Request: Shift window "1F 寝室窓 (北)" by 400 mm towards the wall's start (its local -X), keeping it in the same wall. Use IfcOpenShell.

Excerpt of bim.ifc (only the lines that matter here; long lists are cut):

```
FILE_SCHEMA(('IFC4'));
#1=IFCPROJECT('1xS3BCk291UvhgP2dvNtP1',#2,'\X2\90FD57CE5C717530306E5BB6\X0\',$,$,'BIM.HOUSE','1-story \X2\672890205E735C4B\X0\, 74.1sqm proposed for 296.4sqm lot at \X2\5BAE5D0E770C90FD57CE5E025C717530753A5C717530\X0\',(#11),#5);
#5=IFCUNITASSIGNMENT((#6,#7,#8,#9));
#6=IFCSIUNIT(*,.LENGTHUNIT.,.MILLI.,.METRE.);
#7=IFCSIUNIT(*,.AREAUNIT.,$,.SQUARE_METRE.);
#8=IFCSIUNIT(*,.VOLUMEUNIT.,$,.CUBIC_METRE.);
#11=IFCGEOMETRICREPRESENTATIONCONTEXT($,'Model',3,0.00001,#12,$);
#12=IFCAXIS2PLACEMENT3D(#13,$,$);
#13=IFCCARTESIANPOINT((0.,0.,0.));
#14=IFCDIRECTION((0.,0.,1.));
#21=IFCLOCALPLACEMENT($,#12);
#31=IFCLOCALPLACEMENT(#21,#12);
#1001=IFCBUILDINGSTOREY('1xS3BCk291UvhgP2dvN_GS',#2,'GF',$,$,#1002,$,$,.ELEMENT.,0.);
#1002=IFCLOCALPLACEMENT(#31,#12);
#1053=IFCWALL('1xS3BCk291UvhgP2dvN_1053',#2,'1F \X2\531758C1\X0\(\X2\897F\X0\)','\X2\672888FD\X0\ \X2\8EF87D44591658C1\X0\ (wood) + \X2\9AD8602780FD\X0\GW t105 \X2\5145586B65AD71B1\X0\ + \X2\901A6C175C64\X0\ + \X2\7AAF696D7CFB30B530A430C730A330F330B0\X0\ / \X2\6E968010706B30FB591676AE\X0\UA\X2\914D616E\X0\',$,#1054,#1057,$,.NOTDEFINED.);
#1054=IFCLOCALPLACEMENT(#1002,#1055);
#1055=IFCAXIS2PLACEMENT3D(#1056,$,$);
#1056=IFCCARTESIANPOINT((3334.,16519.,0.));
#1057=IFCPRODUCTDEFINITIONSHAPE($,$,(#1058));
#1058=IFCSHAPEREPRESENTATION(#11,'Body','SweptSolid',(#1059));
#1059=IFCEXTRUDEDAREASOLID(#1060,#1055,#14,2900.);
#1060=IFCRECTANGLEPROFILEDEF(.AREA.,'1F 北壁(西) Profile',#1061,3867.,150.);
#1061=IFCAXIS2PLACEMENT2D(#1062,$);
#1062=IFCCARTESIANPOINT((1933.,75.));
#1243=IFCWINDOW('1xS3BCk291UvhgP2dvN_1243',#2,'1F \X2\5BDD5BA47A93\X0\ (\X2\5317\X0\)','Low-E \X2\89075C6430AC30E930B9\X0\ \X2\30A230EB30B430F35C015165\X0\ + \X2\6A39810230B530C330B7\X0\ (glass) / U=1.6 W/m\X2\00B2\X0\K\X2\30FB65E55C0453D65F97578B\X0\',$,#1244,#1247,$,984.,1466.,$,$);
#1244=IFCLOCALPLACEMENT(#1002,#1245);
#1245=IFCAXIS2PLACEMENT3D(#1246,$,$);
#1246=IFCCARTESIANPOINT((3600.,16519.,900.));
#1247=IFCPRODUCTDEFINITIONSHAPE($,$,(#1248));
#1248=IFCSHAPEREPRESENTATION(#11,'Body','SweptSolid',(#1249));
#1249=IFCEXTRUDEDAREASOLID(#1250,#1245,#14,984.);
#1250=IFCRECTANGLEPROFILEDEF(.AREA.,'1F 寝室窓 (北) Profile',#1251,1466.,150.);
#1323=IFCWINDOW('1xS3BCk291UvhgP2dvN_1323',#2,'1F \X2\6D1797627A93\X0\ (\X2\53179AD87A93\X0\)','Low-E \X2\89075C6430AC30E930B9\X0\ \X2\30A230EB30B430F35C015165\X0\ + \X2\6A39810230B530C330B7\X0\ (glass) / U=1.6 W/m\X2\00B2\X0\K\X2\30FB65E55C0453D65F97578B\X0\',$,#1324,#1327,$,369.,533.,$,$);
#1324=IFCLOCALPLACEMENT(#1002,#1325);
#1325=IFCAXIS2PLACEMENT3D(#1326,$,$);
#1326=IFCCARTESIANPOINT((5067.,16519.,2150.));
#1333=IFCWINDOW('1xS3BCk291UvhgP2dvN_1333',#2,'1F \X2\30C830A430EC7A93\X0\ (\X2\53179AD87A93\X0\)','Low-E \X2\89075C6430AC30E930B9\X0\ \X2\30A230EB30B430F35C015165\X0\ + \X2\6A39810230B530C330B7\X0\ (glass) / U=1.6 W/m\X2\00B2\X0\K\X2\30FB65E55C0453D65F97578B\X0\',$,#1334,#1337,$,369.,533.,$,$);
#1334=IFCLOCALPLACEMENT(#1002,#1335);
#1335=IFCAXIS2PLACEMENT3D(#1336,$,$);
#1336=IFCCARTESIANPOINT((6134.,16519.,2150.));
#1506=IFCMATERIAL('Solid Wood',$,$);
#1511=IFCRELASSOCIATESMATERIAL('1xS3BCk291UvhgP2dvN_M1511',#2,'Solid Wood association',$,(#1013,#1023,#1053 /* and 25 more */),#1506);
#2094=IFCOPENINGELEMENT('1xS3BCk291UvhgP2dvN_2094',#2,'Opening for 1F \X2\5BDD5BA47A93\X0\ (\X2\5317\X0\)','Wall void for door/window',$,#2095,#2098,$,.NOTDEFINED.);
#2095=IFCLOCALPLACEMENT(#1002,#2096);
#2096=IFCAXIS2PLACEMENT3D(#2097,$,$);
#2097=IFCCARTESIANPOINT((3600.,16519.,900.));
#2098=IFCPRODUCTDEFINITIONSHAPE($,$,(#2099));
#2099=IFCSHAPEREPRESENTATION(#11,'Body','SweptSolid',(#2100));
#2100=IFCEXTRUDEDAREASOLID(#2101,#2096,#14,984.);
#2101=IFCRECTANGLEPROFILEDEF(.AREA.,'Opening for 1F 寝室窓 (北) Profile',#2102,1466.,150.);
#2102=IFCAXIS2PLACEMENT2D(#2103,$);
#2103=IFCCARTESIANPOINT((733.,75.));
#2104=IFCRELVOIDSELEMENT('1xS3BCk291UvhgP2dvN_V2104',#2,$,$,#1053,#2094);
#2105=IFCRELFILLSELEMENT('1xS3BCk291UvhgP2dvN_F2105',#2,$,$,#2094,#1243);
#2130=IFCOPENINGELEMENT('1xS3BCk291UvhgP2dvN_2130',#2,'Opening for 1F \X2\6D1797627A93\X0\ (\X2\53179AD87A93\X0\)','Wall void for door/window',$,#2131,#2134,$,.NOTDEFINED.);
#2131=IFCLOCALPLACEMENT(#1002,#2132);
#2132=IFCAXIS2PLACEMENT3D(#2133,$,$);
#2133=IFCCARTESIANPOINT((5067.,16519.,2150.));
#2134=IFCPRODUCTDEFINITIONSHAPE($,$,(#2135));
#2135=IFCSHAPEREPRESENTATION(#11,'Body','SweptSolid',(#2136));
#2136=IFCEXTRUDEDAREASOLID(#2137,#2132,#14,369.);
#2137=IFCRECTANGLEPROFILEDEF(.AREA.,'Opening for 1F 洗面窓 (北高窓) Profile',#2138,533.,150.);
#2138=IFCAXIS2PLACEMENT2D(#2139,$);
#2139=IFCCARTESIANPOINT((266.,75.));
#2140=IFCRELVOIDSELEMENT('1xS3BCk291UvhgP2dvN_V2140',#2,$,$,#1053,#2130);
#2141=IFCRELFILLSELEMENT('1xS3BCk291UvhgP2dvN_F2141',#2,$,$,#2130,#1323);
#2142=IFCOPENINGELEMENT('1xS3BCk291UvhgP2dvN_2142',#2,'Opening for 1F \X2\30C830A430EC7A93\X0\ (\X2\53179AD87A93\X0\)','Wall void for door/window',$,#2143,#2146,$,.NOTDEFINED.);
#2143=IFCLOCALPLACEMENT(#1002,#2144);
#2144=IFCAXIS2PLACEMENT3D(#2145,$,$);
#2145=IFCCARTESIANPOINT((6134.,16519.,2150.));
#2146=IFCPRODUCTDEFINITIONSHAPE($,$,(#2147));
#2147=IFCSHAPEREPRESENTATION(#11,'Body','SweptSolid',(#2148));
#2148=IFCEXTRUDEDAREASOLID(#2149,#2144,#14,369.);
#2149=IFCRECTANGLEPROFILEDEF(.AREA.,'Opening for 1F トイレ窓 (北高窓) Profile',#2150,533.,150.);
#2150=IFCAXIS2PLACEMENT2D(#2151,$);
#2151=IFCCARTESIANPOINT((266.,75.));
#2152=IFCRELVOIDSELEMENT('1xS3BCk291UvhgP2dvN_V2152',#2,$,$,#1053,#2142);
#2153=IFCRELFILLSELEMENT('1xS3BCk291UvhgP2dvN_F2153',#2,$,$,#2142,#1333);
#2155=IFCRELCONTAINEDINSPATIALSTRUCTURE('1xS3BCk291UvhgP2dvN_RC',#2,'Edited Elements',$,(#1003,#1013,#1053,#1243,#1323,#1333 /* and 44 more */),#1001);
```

```python
import ifcopenshell
import ifcopenshell.api.geometry
import ifcopenshell.util.placement
import ifcopenshell.util.unit

model = ifcopenshell.open("bim.ifc")
unit_scale = ifcopenshell.util.unit.calculate_unit_scale(model)

window = model.by_guid("1xS3BCk291UvhgP2dvN_1243")
opening = window.FillsVoids[0].RelatingOpeningElement
wall = opening.VoidsElements[0].RelatingBuildingElement

wall_matrix = ifcopenshell.util.placement.get_local_placement(wall.ObjectPlacement)
shift = wall_matrix[:3, 0] * -0.4 / unit_scale
before = ifcopenshell.util.placement.get_local_placement(window.ObjectPlacement)[:3, 3].copy()

# The window is not placed relative to its opening, so move both.
for product in (opening, window):
    matrix = ifcopenshell.util.placement.get_local_placement(product.ObjectPlacement)
    matrix[:3, 3] += shift
    ifcopenshell.api.geometry.edit_object_placement(model, product=product, matrix=matrix, is_si=False)

after = ifcopenshell.util.placement.get_local_placement(window.ObjectPlacement)[:3, 3]
print("window moved by", (after - before).round(3) + 0.0)

model.write("bim-out.ifc")
```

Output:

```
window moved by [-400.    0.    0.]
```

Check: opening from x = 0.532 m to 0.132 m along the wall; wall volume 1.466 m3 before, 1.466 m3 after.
